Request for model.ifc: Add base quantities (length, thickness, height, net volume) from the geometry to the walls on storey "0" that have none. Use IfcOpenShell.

First a look at what the model holds.

```python
import ifcopenshell
import ifcopenshell.util.element
import ifcopenshell.util.unit

model = ifcopenshell.open("model.ifc")
print(model.schema)
for unit_type in ("LENGTHUNIT", "AREAUNIT", "VOLUMEUNIT"):
    print(unit_type, ifcopenshell.util.unit.calculate_unit_scale(model, unit_type))
storey = next(s for s in model.by_type("IfcBuildingStorey") if s.Name == "0")
walls = [e for e in ifcopenshell.util.element.get_decomposition(storey) if e.is_a("IfcWall")]
for e in sorted(walls, key=lambda e: e.id()):
    print(e.id(), e.is_a(), e.Name, list(ifcopenshell.util.element.get_psets(e, qtos_only=True)), sep=" | ")
```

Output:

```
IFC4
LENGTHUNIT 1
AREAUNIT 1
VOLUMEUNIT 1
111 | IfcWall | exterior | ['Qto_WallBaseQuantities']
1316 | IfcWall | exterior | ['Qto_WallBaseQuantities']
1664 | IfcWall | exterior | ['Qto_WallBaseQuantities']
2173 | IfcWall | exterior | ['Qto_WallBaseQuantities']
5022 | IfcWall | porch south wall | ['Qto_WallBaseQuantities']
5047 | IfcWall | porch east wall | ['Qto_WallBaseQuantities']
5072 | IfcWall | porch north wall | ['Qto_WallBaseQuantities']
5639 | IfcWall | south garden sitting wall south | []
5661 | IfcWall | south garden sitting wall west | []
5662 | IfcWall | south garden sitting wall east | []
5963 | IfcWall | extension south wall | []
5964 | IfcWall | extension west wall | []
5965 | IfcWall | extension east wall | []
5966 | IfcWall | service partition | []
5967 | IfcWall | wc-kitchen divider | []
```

```python
import ifcopenshell
import ifcopenshell.api.pset
import ifcopenshell.geom
import ifcopenshell.util.element
import ifcopenshell.util.shape
import ifcopenshell.util.unit

model = ifcopenshell.open("model.ifc")
unit_scale = ifcopenshell.util.unit.calculate_unit_scale(model)
volume_scale = ifcopenshell.util.unit.calculate_unit_scale(model, "VOLUMEUNIT")
settings = ifcopenshell.geom.settings()

storey = next(s for s in model.by_type("IfcBuildingStorey") if s.Name == "0")
walls = [e for e in ifcopenshell.util.element.get_decomposition(storey) if e.is_a("IfcWall")]

for e in sorted(walls, key=lambda e: e.id()):
    if ifcopenshell.util.element.get_psets(e, qtos_only=True, should_inherit=False):
        continue
    # Geometry comes back in metres, in the element's own axes.
    shape = ifcopenshell.geom.create_shape(settings, e)
    values = {
        "Length": ifcopenshell.util.shape.get_x(shape.geometry) / unit_scale,
        "Width": ifcopenshell.util.shape.get_y(shape.geometry) / unit_scale,
        "Height": ifcopenshell.util.shape.get_z(shape.geometry) / unit_scale,
        "NetVolume": ifcopenshell.util.shape.get_volume(shape.geometry) / volume_scale,
    }
    qto = ifcopenshell.api.pset.add_qto(model, product=e, name="Qto_WallBaseQuantities")
    ifcopenshell.api.pset.edit_qto(model, qto=qto, properties=values)
    print(e.id(), {k: round(v, 3) for k, v in values.items()})

model.write("model_edited.ifc")
```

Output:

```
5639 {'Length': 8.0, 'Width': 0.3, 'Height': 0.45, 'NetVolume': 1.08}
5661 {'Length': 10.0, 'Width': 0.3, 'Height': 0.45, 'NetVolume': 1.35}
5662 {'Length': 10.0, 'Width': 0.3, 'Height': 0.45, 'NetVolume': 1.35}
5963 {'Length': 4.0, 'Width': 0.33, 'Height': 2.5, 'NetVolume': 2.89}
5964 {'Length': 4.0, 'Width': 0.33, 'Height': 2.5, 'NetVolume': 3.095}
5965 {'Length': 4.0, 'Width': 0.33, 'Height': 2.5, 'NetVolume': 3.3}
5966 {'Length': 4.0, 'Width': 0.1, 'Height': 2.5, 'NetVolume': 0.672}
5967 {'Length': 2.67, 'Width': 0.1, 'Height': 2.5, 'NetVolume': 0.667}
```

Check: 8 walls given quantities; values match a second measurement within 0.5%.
